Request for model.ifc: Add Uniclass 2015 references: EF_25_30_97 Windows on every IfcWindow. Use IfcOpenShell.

First a look at what the model holds.

```python
import ifcopenshell

model = ifcopenshell.open("model.ifc")
print(model.schema)
print("classifications:", [c.Name for c in model.by_type("IfcClassification")])
for ifc_class in ("IfcDoor", "IfcRoof", "IfcStair", "IfcWall", "IfcWindow"):
    print(ifc_class, len(model.by_type(ifc_class)))
```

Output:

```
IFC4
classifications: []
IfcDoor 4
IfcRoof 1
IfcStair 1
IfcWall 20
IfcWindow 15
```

```python
import ifcopenshell
import ifcopenshell.api.classification

model = ifcopenshell.open("model.ifc")

system = ifcopenshell.api.classification.add_classification(model, classification="Uniclass 2015")

codes = {
    "IfcWindow": ("EF_25_30_97", "Windows"),
}
for ifc_class, (code, name) in codes.items():
    products = model.by_type(ifc_class)
    ifcopenshell.api.classification.add_reference(
        model, products=products, classification=system, identification=code, name=name
    )
    print(code, len(products))

model.write("model_rev.ifc")
```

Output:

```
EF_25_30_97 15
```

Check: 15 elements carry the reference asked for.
